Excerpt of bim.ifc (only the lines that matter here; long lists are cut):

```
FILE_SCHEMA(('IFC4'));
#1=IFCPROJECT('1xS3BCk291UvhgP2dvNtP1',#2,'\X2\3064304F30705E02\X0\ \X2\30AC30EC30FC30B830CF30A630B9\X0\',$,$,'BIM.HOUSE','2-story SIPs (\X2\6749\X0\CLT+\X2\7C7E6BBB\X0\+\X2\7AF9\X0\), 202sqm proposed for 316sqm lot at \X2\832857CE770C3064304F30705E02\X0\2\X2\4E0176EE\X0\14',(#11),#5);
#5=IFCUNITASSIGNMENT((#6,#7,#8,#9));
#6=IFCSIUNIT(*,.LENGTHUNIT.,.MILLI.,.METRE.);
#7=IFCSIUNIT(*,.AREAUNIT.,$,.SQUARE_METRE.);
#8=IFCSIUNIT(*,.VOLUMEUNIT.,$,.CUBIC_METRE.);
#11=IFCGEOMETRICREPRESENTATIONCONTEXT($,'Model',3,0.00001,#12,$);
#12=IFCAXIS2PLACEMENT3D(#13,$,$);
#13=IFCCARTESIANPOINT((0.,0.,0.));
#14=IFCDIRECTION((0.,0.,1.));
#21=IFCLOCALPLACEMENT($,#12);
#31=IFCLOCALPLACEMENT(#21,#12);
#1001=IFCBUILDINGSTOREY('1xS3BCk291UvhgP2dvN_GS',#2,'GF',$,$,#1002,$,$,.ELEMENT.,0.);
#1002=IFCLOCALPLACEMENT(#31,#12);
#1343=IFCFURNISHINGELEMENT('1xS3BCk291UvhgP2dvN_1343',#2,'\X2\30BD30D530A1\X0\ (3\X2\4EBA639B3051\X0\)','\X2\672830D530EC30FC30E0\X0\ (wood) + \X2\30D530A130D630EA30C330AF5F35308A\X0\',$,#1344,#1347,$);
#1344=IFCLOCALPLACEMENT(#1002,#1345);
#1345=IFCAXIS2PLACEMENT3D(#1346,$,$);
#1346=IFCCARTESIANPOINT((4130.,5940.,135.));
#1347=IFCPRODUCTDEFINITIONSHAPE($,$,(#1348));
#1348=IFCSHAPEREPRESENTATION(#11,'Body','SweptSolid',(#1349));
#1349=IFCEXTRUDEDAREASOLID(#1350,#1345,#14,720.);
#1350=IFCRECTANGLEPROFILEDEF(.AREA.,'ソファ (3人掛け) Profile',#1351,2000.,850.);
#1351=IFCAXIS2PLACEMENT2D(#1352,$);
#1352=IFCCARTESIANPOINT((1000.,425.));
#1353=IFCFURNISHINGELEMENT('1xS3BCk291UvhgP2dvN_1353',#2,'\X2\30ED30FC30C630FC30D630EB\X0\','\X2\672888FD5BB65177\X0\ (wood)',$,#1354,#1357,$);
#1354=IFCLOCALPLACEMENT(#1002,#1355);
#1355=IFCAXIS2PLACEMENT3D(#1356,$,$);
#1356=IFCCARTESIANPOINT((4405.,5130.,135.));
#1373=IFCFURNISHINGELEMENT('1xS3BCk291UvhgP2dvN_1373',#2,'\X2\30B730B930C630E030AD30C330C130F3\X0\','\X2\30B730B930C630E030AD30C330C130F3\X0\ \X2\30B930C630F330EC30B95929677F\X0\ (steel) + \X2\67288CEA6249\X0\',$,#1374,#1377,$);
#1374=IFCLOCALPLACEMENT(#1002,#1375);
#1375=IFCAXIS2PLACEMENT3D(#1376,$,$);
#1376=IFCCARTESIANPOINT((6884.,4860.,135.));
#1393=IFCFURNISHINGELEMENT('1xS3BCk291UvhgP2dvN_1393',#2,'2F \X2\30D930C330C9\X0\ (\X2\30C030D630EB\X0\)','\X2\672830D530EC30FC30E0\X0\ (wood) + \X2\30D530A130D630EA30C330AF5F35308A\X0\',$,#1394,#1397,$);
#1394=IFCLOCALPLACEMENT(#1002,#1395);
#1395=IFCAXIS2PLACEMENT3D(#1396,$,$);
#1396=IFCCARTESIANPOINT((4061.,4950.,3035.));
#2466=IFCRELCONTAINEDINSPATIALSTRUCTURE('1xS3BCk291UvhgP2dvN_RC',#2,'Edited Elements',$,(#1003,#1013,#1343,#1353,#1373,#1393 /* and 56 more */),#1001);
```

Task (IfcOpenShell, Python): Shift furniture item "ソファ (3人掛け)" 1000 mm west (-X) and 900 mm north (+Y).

```python
import ifcopenshell
import ifcopenshell.api.geometry
import ifcopenshell.util.placement

model = ifcopenshell.open("bim.ifc")

item = model.by_id(1343)
matrix = ifcopenshell.util.placement.get_local_placement(item.ObjectPlacement)
matrix[0, 3] -= 1000.0
matrix[1, 3] += 900.0
ifcopenshell.api.geometry.edit_object_placement(model, product=item, matrix=matrix, is_si=False)

print(ifcopenshell.util.placement.get_local_placement(item.ObjectPlacement).round(3) + 0.0)

model.write("bim_v2.ifc")
```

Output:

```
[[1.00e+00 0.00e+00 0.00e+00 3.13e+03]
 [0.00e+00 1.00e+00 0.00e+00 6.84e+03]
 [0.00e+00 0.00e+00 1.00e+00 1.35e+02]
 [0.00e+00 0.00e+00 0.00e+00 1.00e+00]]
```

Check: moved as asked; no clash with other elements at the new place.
